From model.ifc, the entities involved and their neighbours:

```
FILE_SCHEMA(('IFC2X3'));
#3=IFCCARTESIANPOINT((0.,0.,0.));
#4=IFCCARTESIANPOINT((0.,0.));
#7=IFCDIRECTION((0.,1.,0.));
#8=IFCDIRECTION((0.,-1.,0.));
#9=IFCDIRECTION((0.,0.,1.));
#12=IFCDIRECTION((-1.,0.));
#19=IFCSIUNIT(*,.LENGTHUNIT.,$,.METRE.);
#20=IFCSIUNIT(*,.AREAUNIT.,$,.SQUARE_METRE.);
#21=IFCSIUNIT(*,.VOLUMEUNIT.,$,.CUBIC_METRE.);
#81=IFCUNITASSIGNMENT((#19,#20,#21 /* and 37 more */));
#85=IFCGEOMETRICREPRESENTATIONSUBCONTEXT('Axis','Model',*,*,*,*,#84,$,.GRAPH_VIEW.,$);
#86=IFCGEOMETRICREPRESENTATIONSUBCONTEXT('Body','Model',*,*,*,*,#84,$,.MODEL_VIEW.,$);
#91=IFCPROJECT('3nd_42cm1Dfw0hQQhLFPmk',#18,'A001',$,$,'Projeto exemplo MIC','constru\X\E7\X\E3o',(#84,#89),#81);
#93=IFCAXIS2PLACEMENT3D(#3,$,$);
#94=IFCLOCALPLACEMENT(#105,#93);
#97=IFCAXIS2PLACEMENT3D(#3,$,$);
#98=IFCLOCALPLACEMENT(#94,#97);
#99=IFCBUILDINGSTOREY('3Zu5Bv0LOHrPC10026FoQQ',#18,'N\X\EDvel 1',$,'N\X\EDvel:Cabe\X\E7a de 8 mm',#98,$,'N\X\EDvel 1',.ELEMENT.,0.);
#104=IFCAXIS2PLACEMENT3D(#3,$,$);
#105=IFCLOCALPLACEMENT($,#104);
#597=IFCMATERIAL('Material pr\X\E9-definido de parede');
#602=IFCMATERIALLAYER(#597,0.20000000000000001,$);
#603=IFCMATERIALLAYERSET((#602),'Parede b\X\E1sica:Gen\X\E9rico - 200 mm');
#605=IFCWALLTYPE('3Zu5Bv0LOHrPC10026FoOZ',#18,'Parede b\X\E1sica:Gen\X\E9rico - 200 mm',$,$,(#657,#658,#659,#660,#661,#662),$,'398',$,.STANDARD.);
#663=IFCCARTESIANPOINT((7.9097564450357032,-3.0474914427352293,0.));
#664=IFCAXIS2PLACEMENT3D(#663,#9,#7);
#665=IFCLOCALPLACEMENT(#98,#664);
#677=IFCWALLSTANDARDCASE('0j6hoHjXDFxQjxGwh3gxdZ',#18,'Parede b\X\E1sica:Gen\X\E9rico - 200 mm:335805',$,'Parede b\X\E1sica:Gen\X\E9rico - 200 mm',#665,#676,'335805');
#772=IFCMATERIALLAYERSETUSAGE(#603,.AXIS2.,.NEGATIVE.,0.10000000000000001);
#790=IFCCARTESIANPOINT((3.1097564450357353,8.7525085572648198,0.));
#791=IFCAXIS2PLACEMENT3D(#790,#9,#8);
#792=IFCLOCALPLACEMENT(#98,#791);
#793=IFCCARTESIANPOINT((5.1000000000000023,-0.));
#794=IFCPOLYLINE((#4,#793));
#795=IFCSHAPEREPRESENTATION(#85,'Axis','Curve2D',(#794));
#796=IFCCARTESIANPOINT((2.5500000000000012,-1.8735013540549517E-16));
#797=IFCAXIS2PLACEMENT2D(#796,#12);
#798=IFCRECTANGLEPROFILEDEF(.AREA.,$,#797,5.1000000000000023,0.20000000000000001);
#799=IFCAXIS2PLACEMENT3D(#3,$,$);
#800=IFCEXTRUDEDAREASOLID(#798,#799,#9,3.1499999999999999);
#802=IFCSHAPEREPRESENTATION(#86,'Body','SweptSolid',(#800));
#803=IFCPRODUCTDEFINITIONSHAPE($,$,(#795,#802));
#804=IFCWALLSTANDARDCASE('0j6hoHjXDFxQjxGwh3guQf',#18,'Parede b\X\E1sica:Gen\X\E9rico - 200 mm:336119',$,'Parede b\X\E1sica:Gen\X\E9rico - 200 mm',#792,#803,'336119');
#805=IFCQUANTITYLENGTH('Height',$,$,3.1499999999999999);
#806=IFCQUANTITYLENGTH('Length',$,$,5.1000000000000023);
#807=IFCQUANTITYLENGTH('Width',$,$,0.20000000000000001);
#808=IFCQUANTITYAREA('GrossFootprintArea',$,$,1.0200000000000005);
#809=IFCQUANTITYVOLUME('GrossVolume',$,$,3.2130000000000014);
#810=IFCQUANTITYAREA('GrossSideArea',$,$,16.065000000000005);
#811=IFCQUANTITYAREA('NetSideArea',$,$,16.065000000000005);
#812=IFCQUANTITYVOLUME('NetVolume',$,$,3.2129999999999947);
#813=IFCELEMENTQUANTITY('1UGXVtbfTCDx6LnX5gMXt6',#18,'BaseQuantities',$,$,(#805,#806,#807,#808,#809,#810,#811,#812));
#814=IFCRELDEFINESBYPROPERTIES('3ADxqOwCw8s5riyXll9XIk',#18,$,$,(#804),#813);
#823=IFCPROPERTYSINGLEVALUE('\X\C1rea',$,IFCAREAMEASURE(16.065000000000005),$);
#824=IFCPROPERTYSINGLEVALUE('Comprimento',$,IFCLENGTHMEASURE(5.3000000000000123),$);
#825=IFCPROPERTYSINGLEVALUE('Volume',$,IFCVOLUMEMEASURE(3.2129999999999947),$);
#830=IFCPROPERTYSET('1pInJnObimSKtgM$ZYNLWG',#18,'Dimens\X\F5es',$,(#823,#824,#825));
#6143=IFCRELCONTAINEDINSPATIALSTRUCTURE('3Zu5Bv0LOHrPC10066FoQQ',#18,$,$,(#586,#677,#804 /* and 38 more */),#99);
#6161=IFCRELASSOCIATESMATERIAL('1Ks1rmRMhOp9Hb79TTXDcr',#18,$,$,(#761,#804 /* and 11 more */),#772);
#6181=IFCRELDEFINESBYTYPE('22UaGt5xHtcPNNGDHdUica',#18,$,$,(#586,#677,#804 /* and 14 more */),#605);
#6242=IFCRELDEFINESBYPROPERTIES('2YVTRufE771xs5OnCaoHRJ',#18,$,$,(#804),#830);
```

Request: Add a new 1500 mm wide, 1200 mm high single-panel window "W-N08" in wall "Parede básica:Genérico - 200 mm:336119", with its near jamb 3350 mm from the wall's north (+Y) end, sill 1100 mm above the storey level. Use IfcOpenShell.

```python
import numpy as np
import ifcopenshell
import ifcopenshell.api.feature
import ifcopenshell.api.geometry
import ifcopenshell.api.pset
import ifcopenshell.api.root
import ifcopenshell.api.spatial
import ifcopenshell.api.type
import ifcopenshell.geom
import ifcopenshell.util.element
import ifcopenshell.util.placement
import ifcopenshell.util.representation
import ifcopenshell.util.shape
import ifcopenshell.util.unit

model = ifcopenshell.open("model.ifc")
unit_scale = ifcopenshell.util.unit.calculate_unit_scale(model)
area_scale = ifcopenshell.util.unit.calculate_unit_scale(model, "AREAUNIT")
volume_scale = ifcopenshell.util.unit.calculate_unit_scale(model, "VOLUMEUNIT")
settings = ifcopenshell.geom.settings()


def volume(element):
    """Net volume in cubic metres, openings subtracted."""
    shape = ifcopenshell.geom.create_shape(settings, element)
    return ifcopenshell.util.shape.get_volume(shape.geometry)


wall = model.by_id(804)
storey = ifcopenshell.util.element.get_container(wall, ifc_class="IfcBuildingStorey")
context = ifcopenshell.util.representation.get_context(model, "Model", "Body", "MODEL_VIEW")
before = volume(wall)

width, height, from_end, sill = 1.5, 1.2, 3.35, 1.1  # metres

# The wall runs along its own X axis, and the end named is its -X end.
wall_shape = ifcopenshell.geom.create_shape(settings, wall)
x, y, z = ifcopenshell.util.shape.get_vertices(wall_shape.geometry).T
start = x.min() + from_end
face, thickness = float(y.min()), float(y.max() - y.min())
wall_matrix = ifcopenshell.util.placement.get_local_placement(wall.ObjectPlacement)
level = ifcopenshell.util.placement.get_local_placement(storey.ObjectPlacement)[2, 3]


def in_wall(x, y):
    """Placement at x, y metres in the wall's axes, at sill height."""
    matrix = wall_matrix.copy()
    matrix[:, 3] = wall_matrix @ np.array([x / unit_scale, y / unit_scale, 0.0, 1.0])
    matrix[2, 3] = level + sill / unit_scale
    return matrix


# Opening: a box that overshoots both wall faces by 50 mm.
opening = ifcopenshell.api.root.create_entity(model, ifc_class="IfcOpeningElement")
box = ifcopenshell.api.geometry.add_wall_representation(
    model, context=context, length=width, height=height, thickness=thickness + 0.1
)
ifcopenshell.api.geometry.assign_representation(model, product=opening, representation=box)
ifcopenshell.api.geometry.edit_object_placement(model, product=opening, matrix=in_wall(start, face - 0.05), is_si=False)
ifcopenshell.api.feature.add_feature(model, feature=opening, element=wall)

window = ifcopenshell.api.root.create_entity(model, ifc_class="IfcWindow", name="W-N08")
window.OverallWidth, window.OverallHeight = width / unit_scale, height / unit_scale
body = ifcopenshell.api.geometry.add_window_representation(
    model,
    context=context,
    overall_width=window.OverallWidth,
    overall_height=window.OverallHeight,
    partition_type="SINGLE_PANEL",
)
ifcopenshell.api.geometry.assign_representation(model, product=window, representation=body)
ifcopenshell.api.spatial.assign_container(model, products=[window], relating_structure=storey)
fills = ifcopenshell.api.feature.add_filling(model, opening=opening, element=window)
fills.OwnerHistory = window.OwnerHistory  # required in IFC2X3

# IFC2X3 keeps the operation on the window style.
style = ifcopenshell.api.root.create_entity(model, ifc_class="IfcWindowStyle", name="W-N08")
style.OperationType, style.ConstructionType = "SINGLE_PANEL", "NOTDEFINED"
style.ParameterTakesPrecedence = style.Sizeable = False
ifcopenshell.api.type.assign_type(model, related_objects=[window], relating_type=style)

# Centre the window in the wall's thickness.
ifcopenshell.api.geometry.edit_object_placement(model, product=window, matrix=in_wall(start, face), is_si=False)
window_shape = ifcopenshell.geom.create_shape(settings, window)
depth = ifcopenshell.util.shape.get_vertices(window_shape.geometry)[:, 1]
offset = face + thickness / 2 - (depth.min() + depth.max()) / 2
ifcopenshell.api.geometry.edit_object_placement(model, product=window, matrix=in_wall(start, offset), is_si=False)

after = volume(wall)

# Update the wall's stored quantities.
qto = model.by_id(ifcopenshell.util.element.get_pset(wall, "BaseQuantities", should_inherit=False)["id"])
ifcopenshell.api.pset.edit_qto(model, qto=qto, properties={
    "NetSideArea": after / thickness / area_scale,
    "NetVolume": after / volume_scale,
})
pset = model.by_id(ifcopenshell.util.element.get_pset(wall, "Dimensões", should_inherit=False)["id"])
ifcopenshell.api.pset.edit_pset(model, pset=pset, properties={
    "Área": model.create_entity("IfcAreaMeasure", after / thickness / area_scale),
    "Volume": model.create_entity("IfcVolumeMeasure", after / volume_scale),
})

print(f"wall volume {before:.3f} -> {after:.3f} m3")

model.write("model_v2.ifc")
```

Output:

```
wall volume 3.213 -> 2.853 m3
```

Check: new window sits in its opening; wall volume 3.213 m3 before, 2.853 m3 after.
